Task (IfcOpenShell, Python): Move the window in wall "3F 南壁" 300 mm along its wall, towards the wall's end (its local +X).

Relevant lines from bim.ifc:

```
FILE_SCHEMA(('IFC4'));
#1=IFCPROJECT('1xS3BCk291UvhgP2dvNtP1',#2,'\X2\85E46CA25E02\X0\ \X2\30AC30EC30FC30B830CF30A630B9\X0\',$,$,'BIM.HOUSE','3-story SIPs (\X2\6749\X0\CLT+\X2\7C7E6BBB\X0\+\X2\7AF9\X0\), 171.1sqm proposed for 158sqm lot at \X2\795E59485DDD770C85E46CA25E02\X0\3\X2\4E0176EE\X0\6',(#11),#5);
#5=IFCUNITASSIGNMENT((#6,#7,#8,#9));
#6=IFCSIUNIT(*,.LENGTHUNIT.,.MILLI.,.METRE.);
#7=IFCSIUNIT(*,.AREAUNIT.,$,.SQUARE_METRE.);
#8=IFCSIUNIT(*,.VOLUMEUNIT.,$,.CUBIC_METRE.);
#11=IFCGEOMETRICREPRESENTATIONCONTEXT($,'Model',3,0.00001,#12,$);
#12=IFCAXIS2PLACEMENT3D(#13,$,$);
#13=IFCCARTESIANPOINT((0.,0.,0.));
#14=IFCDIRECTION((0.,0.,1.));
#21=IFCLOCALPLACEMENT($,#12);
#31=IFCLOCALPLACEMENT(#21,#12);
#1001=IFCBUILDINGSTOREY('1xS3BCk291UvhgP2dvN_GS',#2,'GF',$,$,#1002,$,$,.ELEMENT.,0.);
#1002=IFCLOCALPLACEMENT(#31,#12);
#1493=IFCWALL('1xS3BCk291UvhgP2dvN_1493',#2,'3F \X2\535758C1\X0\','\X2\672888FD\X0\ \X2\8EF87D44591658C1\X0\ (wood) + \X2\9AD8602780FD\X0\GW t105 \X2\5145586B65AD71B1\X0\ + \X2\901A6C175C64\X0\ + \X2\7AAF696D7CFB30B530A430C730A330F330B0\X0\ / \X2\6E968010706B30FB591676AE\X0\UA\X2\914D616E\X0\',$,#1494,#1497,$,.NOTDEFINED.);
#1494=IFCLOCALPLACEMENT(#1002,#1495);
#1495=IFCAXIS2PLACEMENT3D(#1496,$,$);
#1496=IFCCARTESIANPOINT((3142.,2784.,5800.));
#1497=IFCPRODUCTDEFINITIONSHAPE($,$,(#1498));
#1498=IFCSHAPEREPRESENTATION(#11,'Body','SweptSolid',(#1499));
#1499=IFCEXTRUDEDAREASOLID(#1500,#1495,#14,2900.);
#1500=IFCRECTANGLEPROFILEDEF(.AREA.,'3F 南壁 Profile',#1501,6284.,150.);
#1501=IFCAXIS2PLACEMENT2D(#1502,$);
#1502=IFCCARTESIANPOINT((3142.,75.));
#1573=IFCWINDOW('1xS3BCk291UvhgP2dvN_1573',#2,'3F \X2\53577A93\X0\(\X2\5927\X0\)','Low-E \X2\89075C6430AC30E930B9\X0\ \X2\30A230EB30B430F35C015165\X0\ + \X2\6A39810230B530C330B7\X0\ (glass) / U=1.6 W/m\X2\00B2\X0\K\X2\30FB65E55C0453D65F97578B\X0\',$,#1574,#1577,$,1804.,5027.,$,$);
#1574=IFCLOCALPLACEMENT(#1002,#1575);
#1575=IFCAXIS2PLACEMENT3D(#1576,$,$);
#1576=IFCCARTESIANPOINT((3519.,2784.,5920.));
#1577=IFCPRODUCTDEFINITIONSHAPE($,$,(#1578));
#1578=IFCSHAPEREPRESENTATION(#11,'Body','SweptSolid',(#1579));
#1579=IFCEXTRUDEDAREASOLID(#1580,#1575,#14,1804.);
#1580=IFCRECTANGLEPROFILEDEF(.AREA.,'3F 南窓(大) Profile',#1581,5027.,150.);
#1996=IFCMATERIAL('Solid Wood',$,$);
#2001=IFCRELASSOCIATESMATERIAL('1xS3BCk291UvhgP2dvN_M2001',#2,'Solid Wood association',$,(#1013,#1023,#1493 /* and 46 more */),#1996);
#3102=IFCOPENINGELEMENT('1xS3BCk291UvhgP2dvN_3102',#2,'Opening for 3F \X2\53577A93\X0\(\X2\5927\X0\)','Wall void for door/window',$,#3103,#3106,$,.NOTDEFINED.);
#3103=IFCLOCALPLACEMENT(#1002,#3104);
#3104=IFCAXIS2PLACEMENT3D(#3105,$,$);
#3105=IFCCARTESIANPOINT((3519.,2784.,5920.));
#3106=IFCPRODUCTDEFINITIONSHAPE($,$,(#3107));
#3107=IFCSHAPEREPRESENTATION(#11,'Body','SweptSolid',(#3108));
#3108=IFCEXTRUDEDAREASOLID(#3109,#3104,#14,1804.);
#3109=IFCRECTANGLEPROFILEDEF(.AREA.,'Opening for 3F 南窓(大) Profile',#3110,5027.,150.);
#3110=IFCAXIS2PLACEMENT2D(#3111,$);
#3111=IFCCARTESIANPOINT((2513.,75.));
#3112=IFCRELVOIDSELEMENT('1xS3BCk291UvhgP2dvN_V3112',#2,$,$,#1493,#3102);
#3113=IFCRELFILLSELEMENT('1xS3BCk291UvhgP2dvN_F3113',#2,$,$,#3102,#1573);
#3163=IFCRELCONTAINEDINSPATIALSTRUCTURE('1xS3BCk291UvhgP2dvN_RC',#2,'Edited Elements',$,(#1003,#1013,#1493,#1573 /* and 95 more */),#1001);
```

```python
import ifcopenshell
import ifcopenshell.api.geometry
import ifcopenshell.util.placement

model = ifcopenshell.open("bim.ifc")

window = model.by_id(1573)
opening = window.FillsVoids[0].RelatingOpeningElement
wall = opening.VoidsElements[0].RelatingBuildingElement

wall_matrix = ifcopenshell.util.placement.get_local_placement(wall.ObjectPlacement)
shift = wall_matrix[:3, 0] * 300.0
before = ifcopenshell.util.placement.get_local_placement(window.ObjectPlacement)[:3, 3].copy()

# The window is not placed relative to its opening, so move both.
for product in (opening, window):
    matrix = ifcopenshell.util.placement.get_local_placement(product.ObjectPlacement)
    matrix[:3, 3] += shift
    ifcopenshell.api.geometry.edit_object_placement(model, product=product, matrix=matrix, is_si=False)

after = ifcopenshell.util.placement.get_local_placement(window.ObjectPlacement)[:3, 3]
print("window moved by", (after - before).round(3) + 0.0)

model.write("bim_v2.ifc")
```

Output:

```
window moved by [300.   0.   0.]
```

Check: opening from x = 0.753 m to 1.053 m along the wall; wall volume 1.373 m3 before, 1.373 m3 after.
